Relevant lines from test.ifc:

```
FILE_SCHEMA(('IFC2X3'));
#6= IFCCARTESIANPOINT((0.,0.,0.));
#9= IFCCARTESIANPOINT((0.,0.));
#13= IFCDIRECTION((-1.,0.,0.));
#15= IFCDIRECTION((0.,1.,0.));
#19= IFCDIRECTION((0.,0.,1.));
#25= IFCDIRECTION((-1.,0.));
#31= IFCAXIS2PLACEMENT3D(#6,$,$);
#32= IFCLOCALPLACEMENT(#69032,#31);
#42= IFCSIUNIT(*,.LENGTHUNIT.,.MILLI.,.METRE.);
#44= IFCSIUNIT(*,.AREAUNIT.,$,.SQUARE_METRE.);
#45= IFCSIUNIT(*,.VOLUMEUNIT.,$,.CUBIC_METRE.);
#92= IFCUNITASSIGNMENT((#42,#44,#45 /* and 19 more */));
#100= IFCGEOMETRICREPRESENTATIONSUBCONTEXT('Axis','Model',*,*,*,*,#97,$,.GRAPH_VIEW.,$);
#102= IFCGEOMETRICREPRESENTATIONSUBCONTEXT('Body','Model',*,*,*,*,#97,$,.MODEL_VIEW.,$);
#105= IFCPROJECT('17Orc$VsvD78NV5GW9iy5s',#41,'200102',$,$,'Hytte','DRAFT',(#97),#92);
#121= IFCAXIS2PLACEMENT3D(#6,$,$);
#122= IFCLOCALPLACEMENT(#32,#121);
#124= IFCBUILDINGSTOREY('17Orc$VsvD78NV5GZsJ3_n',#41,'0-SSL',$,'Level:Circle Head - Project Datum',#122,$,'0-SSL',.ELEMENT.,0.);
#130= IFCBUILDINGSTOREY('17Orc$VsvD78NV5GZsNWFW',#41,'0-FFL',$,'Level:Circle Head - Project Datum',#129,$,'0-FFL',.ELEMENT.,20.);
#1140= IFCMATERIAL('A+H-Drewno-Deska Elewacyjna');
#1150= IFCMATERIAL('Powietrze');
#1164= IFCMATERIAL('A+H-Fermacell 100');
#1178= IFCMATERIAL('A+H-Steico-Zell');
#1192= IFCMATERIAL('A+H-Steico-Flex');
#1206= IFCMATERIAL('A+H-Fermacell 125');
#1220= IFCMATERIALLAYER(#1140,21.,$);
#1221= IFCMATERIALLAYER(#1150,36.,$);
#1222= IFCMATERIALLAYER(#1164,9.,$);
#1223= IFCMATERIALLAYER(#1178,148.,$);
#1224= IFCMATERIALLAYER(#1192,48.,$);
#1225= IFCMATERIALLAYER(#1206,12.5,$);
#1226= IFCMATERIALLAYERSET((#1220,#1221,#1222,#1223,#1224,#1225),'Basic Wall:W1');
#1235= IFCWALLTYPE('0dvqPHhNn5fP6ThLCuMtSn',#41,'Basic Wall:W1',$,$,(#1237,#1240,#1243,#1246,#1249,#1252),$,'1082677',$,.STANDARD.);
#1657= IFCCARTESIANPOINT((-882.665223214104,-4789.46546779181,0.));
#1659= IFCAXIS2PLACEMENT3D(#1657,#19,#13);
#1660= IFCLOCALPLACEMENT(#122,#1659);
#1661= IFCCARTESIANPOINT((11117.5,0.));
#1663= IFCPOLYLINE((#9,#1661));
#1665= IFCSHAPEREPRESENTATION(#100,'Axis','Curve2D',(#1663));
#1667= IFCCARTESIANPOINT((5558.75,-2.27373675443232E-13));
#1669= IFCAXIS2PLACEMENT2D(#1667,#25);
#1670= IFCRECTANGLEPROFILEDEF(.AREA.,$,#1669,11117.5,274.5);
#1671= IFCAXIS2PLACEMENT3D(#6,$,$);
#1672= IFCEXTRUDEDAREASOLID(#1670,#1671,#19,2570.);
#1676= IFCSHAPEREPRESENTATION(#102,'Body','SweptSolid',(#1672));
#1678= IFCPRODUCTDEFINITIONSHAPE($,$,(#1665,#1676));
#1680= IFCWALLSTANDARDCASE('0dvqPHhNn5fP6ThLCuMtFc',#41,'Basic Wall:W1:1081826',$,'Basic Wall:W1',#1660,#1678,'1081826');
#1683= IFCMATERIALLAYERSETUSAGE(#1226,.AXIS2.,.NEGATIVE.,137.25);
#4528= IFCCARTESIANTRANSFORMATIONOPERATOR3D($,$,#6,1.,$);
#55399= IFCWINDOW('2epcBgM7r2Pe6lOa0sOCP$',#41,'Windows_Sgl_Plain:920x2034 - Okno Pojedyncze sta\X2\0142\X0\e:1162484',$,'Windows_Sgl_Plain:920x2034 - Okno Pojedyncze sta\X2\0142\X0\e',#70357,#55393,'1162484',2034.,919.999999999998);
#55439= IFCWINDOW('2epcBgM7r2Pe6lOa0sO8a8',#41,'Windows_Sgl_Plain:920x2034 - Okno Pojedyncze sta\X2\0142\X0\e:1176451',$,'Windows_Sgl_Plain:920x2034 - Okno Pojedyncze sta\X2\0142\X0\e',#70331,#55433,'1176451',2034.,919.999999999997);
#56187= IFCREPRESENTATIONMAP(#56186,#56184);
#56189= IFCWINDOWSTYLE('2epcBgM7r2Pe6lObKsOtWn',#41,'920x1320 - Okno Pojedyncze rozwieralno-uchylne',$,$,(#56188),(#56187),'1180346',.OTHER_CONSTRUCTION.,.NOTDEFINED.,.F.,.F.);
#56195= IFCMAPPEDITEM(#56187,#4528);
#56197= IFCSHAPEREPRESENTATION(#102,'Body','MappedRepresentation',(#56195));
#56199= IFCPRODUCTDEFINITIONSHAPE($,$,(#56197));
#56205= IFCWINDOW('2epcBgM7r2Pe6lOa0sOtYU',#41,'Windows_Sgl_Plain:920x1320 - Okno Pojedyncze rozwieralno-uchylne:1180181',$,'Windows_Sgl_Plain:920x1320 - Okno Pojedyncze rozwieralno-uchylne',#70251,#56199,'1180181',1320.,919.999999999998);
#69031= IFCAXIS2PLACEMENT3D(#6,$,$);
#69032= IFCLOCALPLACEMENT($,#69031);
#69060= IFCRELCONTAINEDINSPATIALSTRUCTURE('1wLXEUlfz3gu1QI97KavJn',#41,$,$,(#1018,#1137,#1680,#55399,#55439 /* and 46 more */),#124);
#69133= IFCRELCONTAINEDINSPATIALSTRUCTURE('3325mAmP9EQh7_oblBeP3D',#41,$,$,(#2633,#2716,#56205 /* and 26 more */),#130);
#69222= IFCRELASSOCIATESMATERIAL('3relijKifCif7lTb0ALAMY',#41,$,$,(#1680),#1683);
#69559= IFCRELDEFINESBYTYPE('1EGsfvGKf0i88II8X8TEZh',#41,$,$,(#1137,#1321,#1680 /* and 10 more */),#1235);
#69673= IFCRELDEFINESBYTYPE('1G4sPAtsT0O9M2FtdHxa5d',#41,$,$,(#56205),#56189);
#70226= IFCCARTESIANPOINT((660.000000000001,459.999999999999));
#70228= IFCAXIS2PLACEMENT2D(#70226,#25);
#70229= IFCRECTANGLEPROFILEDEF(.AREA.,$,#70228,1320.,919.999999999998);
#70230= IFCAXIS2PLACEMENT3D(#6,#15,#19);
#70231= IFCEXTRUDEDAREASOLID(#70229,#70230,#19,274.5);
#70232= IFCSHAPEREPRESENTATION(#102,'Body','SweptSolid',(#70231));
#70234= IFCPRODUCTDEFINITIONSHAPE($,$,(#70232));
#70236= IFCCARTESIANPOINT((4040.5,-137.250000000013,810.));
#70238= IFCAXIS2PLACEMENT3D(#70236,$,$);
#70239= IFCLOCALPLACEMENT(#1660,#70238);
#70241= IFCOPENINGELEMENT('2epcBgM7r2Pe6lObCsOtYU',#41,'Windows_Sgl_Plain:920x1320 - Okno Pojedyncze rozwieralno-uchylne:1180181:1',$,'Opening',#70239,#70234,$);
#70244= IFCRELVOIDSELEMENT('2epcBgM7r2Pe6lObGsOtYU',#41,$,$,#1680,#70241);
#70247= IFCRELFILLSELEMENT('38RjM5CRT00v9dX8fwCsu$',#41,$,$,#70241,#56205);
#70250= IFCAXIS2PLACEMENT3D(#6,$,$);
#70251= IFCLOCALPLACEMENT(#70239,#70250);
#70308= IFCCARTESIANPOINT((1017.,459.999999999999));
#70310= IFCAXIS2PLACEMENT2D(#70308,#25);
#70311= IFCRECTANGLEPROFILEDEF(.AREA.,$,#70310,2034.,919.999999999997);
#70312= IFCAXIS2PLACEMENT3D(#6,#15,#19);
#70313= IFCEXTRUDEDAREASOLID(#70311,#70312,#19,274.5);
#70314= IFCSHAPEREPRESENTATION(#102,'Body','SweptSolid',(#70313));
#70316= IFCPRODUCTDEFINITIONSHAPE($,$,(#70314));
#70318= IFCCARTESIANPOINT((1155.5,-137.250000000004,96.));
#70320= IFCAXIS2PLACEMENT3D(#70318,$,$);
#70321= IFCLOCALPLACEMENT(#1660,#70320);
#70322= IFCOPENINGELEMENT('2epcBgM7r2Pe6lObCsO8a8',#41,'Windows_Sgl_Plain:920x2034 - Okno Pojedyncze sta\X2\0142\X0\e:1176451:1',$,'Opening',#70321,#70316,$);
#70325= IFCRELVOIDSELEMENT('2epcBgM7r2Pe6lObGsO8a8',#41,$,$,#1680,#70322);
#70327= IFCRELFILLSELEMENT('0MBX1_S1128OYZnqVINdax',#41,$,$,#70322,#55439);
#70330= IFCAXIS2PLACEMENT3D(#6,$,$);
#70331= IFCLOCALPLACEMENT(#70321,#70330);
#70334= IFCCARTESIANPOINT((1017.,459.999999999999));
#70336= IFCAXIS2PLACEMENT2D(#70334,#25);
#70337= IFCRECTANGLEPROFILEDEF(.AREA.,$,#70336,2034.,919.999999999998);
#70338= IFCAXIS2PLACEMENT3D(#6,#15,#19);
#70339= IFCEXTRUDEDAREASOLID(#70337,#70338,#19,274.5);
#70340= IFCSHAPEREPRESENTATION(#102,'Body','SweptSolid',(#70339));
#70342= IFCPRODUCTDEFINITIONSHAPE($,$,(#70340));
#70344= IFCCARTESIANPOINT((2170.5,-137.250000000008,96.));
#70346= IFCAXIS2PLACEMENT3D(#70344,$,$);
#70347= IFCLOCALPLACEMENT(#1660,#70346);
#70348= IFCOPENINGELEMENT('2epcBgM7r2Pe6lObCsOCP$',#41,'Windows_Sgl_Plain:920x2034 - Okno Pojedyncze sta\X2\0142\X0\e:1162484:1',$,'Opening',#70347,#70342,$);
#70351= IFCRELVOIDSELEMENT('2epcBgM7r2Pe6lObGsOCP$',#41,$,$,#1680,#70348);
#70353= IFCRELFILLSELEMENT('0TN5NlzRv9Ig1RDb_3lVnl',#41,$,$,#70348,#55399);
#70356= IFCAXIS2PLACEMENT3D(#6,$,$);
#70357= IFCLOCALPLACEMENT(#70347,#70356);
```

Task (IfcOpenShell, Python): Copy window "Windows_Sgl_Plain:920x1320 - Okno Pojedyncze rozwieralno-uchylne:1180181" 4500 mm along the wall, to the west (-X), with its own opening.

```python
import ifcopenshell
import ifcopenshell.api.feature
import ifcopenshell.api.geometry
import ifcopenshell.api.root
import ifcopenshell.geom
import ifcopenshell.util.element
import ifcopenshell.util.placement
import ifcopenshell.util.shape
import ifcopenshell.util.unit

model = ifcopenshell.open("test.ifc")
unit_scale = ifcopenshell.util.unit.calculate_unit_scale(model)
settings = ifcopenshell.geom.settings()


def volume(element):
    """Net volume in cubic metres, openings subtracted."""
    shape = ifcopenshell.geom.create_shape(settings, element)
    return ifcopenshell.util.shape.get_volume(shape.geometry)


def reuse_history(source, copy):
    """copy_class also copies each property set's owner history, people and application; keep the originals."""
    for rel in copy.IsDefinedBy:
        if rel.is_a("IfcRelDefinesByProperties") and (history := rel.RelatingPropertyDefinition.OwnerHistory):
            rel.RelatingPropertyDefinition.OwnerHistory = source.OwnerHistory
            ifcopenshell.util.element.remove_deep2(model, history)


window = model.by_guid("2epcBgM7r2Pe6lOa0sOtYU")
opening = window.FillsVoids[0].RelatingOpeningElement
wall = opening.VoidsElements[0].RelatingBuildingElement
before = volume(wall)
shift = ifcopenshell.util.placement.get_local_placement(wall.ObjectPlacement)[:3, 0] * 4.5 / unit_scale

# copy_class copies the void relationship, type, container and properties, but no geometry.
new_opening = ifcopenshell.api.root.copy_class(model, product=opening)
new_opening.Representation = ifcopenshell.util.element.copy_deep(
    model, opening.Representation, exclude=["IfcGeometricRepresentationContext", "IfcRepresentationMap"]
)
new_opening.Name = "Windows_Sgl_Plain:920x1320 - Okno Pojedyncze rozwieralno-uchylne"
new_window = ifcopenshell.api.root.copy_class(model, product=window)
new_window.Representation = ifcopenshell.util.element.copy_deep(
    model, window.Representation, exclude=["IfcGeometricRepresentationContext", "IfcRepresentationMap"]
)
new_window.Name = "Windows_Sgl_Plain:920x1320 - Okno Pojedyncze rozwieralno-uchylne"
new_window.Tag = None
reuse_history(window, new_window)
fills = ifcopenshell.api.feature.add_filling(model, opening=new_opening, element=new_window)
fills.OwnerHistory = new_window.OwnerHistory  # required in IFC2X3

for old, new in ((opening, new_opening), (window, new_window)):
    matrix = ifcopenshell.util.placement.get_local_placement(old.ObjectPlacement)
    matrix[:3, 3] += shift
    ifcopenshell.api.geometry.edit_object_placement(model, product=new, matrix=matrix, is_si=False)

after = volume(wall)

print(f"wall volume {before:.3f} -> {after:.3f} m3")

model.write("test_updated.ifc")
```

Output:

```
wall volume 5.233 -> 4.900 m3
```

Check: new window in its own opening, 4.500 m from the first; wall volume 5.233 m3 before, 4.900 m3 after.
